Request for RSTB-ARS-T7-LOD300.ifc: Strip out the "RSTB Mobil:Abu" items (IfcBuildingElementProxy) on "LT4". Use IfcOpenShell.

First a look at what the model holds.

```python
import ifcopenshell
import ifcopenshell.util.element

model = ifcopenshell.open("RSTB-ARS-T7-LOD300.ifc")
print(model.schema)
storey = next(s for s in model.by_type("IfcBuildingStorey") if s.Name == "LT4")
proxies = [e for e in ifcopenshell.util.element.get_decomposition(storey) if e.is_a("IfcBuildingElementProxy")]
seen = {}
for e in proxies:
    element_type = ifcopenshell.util.element.get_type(e)
    name = element_type.Name if element_type not in (None, e) else None
    seen[name] = seen.get(name, 0) + 1
for name, count in sorted(seen.items(), key=str):
    print(count, "x", name)
```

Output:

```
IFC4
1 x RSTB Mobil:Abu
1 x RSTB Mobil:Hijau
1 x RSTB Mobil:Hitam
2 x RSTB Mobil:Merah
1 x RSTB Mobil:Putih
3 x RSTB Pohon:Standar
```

```python
import ifcopenshell
import ifcopenshell.api.root
import ifcopenshell.util.element

model = ifcopenshell.open("RSTB-ARS-T7-LOD300.ifc")

storey = next(s for s in model.by_type("IfcBuildingStorey") if s.Name == "LT4")
proxies = [e for e in ifcopenshell.util.element.get_decomposition(storey) if e.is_a("IfcBuildingElementProxy")]
targets = [e for e in proxies if (t := ifcopenshell.util.element.get_type(e)) not in (None, e) and t.Name == "RSTB Mobil:Abu"]

for e in targets:
    ifcopenshell.api.root.remove_product(model, product=e)
print(len(targets), "removed")

model.write("RSTB-ARS-T7-LOD300_edited.ifc")
```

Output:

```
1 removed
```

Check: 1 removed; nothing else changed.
